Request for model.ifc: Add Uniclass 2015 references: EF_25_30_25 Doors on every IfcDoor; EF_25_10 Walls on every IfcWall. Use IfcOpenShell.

First a look at what the model holds.

```python
import ifcopenshell

model = ifcopenshell.open("model.ifc")
print(model.schema)
print("classifications:", [c.Name for c in model.by_type("IfcClassification")])
for ifc_class in ("IfcDoor", "IfcRoof", "IfcStair", "IfcWall", "IfcWindow"):
    print(ifc_class, len(model.by_type(ifc_class)))
```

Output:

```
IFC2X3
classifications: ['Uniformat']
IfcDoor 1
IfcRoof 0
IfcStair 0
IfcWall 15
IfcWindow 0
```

```python
import ifcopenshell
import ifcopenshell.api.classification

model = ifcopenshell.open("model.ifc")

# IFC2X3 requires Source and Edition and has no link from the project to the system.
system = model.create_entity("IfcClassification", Source="NBS", Edition="2015", Name="Uniclass 2015")

codes = {
    "IfcDoor": ("EF_25_30_25", "Doors"),
    "IfcWall": ("EF_25_10", "Walls"),
}
for ifc_class, (code, name) in codes.items():
    products = model.by_type(ifc_class)
    ifcopenshell.api.classification.add_reference(
        model, products=products, classification=system, identification=code, name=name
    )
    print(code, len(products))

model.write("model-out.ifc")
```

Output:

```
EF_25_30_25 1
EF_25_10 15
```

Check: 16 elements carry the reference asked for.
